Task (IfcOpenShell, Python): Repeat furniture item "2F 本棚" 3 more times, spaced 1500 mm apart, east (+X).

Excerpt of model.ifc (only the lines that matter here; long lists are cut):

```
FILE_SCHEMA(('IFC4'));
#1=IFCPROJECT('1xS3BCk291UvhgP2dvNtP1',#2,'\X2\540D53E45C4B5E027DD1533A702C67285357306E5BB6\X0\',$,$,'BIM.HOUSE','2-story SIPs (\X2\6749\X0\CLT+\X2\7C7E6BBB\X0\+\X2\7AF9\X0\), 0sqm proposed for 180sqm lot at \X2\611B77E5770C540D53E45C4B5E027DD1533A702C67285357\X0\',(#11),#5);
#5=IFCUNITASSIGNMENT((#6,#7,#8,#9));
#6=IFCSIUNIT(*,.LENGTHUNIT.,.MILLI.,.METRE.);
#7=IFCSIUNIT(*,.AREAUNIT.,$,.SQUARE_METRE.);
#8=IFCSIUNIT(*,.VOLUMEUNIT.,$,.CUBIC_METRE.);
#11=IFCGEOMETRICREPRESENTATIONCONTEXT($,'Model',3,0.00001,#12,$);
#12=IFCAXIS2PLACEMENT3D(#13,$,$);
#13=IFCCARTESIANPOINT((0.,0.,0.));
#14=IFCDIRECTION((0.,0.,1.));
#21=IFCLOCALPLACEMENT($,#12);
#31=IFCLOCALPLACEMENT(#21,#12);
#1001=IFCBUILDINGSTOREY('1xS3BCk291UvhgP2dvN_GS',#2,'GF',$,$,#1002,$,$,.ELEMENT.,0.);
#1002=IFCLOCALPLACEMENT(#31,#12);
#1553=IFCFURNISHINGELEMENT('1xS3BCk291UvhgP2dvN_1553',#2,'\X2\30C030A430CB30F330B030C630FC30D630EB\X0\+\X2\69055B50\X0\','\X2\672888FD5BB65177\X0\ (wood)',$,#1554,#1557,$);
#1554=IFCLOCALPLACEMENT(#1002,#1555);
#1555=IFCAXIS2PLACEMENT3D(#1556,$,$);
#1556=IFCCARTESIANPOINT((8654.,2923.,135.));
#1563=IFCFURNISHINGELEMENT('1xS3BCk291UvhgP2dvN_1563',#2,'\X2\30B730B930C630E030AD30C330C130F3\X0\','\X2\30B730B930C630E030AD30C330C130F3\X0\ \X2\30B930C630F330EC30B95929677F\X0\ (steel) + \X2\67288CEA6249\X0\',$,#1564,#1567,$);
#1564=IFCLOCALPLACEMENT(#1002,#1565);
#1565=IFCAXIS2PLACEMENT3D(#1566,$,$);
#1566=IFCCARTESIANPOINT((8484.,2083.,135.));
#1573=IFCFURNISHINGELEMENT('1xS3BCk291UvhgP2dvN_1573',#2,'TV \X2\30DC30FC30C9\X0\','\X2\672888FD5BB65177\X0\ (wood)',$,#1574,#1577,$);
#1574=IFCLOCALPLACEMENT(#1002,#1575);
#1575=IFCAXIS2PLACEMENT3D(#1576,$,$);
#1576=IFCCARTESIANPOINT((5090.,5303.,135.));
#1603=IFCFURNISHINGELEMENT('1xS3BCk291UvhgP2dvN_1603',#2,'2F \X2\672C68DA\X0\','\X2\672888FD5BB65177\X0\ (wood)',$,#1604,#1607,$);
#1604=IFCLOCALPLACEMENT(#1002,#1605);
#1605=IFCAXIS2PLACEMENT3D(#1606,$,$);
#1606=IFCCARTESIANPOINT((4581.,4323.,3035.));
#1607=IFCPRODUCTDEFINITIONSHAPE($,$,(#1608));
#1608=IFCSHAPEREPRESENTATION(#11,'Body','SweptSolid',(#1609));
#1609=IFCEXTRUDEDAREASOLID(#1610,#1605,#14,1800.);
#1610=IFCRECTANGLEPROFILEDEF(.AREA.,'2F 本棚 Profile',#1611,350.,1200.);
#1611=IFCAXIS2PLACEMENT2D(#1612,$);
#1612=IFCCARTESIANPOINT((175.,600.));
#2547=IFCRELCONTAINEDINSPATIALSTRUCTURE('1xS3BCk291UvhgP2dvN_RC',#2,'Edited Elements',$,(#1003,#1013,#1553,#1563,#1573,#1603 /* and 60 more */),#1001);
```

```python
import numpy as np
import ifcopenshell
import ifcopenshell.api.geometry
import ifcopenshell.api.root
import ifcopenshell.util.element
import ifcopenshell.util.placement
import ifcopenshell.util.unit

model = ifcopenshell.open("model.ifc")
unit_scale = ifcopenshell.util.unit.calculate_unit_scale(model)


def reuse_history(source, copy):
    """copy_class also copies each property set's owner history, people and application; keep the originals."""
    for rel in copy.IsDefinedBy:
        if rel.is_a("IfcRelDefinesByProperties") and (history := rel.RelatingPropertyDefinition.OwnerHistory):
            rel.RelatingPropertyDefinition.OwnerHistory = source.OwnerHistory
            ifcopenshell.util.element.remove_deep2(model, history)


source = model.by_guid("1xS3BCk291UvhgP2dvN_1603")
base = ifcopenshell.util.placement.get_local_placement(source.ObjectPlacement)
step = np.array([1.0, 0.0, 0.0]) * 1.5 / unit_scale

for i in range(1, 4):
    copy = ifcopenshell.api.root.copy_class(model, product=source)
    copy.Representation = ifcopenshell.util.element.copy_deep(
        model, source.Representation, exclude=["IfcGeometricRepresentationContext", "IfcRepresentationMap"]
    )
    reuse_history(source, copy)
    matrix = base.copy()
    matrix[:3, 3] += i * step
    print("added at", matrix[:3, 3].round(3) + 0.0)
    ifcopenshell.api.geometry.edit_object_placement(model, product=copy, matrix=matrix, is_si=False)

model.write("model_updated.ifc")
```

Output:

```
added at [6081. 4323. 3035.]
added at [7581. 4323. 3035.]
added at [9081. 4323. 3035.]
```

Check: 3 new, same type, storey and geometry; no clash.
